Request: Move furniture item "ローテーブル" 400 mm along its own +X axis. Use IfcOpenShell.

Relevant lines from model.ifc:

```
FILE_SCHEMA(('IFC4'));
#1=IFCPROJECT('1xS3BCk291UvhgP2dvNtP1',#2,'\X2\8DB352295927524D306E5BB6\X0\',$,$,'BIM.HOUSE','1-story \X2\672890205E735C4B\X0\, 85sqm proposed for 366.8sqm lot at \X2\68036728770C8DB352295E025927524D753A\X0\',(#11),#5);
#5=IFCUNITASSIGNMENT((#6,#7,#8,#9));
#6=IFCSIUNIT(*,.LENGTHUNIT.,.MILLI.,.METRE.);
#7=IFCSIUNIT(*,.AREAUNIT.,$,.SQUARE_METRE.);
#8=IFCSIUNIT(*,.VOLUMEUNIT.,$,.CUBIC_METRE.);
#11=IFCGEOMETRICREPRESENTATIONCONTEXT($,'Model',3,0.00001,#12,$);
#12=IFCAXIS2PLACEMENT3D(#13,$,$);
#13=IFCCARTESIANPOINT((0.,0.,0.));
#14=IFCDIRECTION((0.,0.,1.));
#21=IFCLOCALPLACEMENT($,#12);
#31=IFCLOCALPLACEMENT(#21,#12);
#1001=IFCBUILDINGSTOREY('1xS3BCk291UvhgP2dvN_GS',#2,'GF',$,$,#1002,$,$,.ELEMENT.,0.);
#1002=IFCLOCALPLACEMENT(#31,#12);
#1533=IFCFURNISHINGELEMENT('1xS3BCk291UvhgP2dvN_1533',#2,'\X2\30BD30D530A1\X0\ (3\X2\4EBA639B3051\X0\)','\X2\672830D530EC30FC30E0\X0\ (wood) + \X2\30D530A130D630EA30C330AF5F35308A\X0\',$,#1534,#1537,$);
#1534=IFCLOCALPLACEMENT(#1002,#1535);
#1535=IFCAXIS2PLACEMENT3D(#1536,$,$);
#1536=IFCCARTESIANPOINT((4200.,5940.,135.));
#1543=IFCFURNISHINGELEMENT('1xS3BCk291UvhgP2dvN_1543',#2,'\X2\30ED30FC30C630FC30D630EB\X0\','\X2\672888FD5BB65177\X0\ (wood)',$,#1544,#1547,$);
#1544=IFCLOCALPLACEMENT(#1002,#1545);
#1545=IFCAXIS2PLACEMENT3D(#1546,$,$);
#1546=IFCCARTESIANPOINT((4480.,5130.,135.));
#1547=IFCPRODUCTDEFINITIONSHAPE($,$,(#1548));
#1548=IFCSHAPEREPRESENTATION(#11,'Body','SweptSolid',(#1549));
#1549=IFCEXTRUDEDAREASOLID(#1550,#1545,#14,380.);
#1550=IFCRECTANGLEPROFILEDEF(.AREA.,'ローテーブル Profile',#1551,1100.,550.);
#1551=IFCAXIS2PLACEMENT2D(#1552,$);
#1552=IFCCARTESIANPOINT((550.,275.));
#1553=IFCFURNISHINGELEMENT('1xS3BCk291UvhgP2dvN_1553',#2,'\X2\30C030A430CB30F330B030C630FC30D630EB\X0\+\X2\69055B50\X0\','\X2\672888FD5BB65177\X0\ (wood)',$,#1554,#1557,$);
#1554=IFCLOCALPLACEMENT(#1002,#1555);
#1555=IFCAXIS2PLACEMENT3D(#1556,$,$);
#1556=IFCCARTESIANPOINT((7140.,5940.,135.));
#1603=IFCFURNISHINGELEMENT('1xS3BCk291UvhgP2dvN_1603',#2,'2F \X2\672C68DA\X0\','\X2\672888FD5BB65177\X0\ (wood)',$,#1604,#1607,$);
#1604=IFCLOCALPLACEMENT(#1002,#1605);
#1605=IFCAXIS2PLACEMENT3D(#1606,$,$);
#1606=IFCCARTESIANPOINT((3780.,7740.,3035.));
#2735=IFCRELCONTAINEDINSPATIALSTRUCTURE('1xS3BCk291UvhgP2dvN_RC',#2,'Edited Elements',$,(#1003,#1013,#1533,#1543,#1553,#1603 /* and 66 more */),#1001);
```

```python
import ifcopenshell
import ifcopenshell.api.geometry
import ifcopenshell.util.placement
import ifcopenshell.util.unit

model = ifcopenshell.open("model.ifc")
unit_scale = ifcopenshell.util.unit.calculate_unit_scale(model)

item = model.by_guid("1xS3BCk291UvhgP2dvN_1543")
matrix = ifcopenshell.util.placement.get_local_placement(item.ObjectPlacement)
matrix[:3, 3] += matrix[:3, 0] * 0.4 / unit_scale
ifcopenshell.api.geometry.edit_object_placement(model, product=item, matrix=matrix, is_si=False)

print(ifcopenshell.util.placement.get_local_placement(item.ObjectPlacement).round(3) + 0.0)

model.write("model_rev.ifc")
```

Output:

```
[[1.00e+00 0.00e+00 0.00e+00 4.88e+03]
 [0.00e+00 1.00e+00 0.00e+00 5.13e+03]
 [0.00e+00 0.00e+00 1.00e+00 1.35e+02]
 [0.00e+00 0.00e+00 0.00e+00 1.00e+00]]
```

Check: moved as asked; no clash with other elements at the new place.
